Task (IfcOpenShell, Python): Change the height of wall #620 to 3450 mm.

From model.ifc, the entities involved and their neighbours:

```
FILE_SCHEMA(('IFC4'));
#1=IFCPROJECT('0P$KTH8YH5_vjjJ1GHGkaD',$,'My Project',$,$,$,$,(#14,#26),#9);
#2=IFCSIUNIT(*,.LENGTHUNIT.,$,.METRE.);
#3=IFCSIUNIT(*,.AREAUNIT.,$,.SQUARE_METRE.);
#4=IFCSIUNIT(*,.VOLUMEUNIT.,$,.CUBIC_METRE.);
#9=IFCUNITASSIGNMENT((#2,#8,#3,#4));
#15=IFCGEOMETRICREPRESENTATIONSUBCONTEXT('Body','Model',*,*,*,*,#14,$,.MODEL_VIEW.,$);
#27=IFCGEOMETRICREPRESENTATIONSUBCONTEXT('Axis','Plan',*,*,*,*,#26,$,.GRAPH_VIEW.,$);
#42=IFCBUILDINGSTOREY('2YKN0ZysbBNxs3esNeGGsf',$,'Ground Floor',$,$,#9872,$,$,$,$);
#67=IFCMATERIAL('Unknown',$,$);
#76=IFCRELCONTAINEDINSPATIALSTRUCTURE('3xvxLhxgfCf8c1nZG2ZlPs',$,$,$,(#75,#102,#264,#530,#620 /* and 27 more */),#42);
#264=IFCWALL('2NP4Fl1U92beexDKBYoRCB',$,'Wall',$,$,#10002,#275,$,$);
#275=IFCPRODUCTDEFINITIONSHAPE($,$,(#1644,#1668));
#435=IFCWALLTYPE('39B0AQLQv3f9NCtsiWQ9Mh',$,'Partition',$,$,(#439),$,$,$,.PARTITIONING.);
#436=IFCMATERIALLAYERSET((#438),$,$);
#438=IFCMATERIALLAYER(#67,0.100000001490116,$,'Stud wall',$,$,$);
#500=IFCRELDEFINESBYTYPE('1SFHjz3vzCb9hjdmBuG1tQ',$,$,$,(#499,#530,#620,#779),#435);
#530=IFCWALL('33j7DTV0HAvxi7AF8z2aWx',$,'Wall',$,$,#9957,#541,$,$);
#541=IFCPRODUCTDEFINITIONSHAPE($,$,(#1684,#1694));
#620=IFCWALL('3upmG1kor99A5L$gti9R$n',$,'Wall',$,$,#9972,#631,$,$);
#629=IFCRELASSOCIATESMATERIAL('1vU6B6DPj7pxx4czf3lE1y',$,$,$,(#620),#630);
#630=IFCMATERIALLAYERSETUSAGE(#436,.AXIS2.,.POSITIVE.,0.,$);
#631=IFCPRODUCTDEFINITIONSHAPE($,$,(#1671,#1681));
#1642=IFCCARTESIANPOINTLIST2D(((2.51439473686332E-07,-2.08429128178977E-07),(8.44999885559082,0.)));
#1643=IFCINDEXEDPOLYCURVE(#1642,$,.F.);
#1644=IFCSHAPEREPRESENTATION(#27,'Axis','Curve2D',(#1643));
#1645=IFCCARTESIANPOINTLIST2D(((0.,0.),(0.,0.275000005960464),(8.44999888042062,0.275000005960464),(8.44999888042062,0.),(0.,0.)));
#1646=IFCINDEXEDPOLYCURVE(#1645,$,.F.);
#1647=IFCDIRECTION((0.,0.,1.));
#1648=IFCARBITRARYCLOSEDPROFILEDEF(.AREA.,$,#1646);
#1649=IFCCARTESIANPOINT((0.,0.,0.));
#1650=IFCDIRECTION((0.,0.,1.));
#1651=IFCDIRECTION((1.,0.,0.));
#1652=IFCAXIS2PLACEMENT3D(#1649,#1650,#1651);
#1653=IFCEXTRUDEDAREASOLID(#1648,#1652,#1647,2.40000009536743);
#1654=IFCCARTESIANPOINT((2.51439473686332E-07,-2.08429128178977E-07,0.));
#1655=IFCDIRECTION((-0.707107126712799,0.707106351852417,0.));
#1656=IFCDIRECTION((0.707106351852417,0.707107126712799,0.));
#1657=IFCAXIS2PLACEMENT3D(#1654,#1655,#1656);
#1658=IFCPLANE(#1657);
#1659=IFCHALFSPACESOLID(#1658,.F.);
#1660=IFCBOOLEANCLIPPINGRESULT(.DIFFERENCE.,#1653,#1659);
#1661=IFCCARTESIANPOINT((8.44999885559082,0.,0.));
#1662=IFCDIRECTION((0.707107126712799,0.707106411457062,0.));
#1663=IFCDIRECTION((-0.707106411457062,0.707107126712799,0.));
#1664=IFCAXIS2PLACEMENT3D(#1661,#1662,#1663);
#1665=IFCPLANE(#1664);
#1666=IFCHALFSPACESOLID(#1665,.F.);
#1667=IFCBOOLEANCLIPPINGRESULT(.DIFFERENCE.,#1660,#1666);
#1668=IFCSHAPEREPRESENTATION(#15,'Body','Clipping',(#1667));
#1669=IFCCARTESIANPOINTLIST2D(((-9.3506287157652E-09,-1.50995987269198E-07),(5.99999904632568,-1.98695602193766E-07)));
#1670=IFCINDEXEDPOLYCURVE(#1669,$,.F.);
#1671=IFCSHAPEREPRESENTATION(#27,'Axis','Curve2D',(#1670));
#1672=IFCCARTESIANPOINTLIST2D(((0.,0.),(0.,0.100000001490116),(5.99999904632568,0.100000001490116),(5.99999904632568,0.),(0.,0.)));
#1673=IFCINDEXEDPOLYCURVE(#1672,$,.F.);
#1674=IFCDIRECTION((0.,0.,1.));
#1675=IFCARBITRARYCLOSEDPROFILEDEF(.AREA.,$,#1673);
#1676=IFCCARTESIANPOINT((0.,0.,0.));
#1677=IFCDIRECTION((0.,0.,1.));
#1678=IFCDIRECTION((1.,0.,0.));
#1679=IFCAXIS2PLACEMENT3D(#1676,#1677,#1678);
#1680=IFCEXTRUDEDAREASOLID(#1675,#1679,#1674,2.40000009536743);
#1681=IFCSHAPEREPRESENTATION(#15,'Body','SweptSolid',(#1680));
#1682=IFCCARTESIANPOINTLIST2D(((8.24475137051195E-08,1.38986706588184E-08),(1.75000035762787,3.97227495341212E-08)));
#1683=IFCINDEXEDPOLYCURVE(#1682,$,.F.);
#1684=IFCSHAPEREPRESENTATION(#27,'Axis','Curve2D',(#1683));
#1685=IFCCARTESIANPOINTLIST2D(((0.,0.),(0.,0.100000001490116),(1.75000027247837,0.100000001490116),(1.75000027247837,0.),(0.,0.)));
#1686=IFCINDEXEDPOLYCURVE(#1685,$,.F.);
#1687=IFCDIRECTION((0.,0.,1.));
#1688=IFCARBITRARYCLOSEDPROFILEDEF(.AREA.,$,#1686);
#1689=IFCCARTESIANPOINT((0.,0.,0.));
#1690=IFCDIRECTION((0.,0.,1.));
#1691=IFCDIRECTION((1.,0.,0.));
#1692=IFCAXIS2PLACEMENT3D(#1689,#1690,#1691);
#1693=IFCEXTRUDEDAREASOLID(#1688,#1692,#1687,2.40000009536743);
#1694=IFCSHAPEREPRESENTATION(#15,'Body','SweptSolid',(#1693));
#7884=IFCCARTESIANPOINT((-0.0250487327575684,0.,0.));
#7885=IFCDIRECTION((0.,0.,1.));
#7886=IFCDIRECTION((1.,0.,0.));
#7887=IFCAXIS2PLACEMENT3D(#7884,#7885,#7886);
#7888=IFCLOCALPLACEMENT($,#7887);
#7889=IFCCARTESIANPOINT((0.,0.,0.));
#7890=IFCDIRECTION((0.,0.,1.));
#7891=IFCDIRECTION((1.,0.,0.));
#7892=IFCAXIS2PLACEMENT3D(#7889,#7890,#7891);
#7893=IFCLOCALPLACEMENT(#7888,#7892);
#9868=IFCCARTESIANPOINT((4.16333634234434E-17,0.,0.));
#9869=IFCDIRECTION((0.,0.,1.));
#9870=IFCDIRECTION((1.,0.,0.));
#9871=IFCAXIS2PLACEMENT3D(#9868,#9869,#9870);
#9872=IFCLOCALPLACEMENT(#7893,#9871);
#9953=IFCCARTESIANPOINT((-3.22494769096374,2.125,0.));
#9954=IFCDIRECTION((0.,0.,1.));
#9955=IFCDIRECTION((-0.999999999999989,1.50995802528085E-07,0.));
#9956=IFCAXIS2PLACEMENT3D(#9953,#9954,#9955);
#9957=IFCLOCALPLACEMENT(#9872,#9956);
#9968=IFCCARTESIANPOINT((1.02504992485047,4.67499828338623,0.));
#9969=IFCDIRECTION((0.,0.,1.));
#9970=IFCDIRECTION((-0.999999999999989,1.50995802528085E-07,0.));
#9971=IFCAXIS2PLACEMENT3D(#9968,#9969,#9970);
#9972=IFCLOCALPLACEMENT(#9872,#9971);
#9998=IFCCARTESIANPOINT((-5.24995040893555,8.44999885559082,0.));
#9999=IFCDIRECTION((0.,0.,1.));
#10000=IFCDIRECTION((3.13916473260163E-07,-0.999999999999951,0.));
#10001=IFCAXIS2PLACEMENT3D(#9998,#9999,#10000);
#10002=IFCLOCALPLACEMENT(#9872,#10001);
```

```python
import ifcopenshell
import ifcopenshell.geom
import ifcopenshell.util.representation
import ifcopenshell.util.shape

model = ifcopenshell.open("model.ifc")
settings = ifcopenshell.geom.settings()


def volume(element):
    """Net volume in cubic metres, openings subtracted."""
    shape = ifcopenshell.geom.create_shape(settings, element)
    return ifcopenshell.util.shape.get_volume(shape.geometry)


wall = model.by_guid("3upmG1kor99A5L$gti9R$n")
before = volume(wall)

body = ifcopenshell.util.representation.get_representation(wall, "Model", "Body")
solid = body.Items[0]
old_height = solid.Depth
solid.Depth = 3.45
after = volume(wall)

print(f"height {old_height:g} -> {solid.Depth:g}, volume {before:.3f} -> {after:.3f} m3")

model.write("model_v2.ifc")
```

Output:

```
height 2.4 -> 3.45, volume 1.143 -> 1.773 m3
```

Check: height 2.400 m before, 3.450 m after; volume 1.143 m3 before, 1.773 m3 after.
